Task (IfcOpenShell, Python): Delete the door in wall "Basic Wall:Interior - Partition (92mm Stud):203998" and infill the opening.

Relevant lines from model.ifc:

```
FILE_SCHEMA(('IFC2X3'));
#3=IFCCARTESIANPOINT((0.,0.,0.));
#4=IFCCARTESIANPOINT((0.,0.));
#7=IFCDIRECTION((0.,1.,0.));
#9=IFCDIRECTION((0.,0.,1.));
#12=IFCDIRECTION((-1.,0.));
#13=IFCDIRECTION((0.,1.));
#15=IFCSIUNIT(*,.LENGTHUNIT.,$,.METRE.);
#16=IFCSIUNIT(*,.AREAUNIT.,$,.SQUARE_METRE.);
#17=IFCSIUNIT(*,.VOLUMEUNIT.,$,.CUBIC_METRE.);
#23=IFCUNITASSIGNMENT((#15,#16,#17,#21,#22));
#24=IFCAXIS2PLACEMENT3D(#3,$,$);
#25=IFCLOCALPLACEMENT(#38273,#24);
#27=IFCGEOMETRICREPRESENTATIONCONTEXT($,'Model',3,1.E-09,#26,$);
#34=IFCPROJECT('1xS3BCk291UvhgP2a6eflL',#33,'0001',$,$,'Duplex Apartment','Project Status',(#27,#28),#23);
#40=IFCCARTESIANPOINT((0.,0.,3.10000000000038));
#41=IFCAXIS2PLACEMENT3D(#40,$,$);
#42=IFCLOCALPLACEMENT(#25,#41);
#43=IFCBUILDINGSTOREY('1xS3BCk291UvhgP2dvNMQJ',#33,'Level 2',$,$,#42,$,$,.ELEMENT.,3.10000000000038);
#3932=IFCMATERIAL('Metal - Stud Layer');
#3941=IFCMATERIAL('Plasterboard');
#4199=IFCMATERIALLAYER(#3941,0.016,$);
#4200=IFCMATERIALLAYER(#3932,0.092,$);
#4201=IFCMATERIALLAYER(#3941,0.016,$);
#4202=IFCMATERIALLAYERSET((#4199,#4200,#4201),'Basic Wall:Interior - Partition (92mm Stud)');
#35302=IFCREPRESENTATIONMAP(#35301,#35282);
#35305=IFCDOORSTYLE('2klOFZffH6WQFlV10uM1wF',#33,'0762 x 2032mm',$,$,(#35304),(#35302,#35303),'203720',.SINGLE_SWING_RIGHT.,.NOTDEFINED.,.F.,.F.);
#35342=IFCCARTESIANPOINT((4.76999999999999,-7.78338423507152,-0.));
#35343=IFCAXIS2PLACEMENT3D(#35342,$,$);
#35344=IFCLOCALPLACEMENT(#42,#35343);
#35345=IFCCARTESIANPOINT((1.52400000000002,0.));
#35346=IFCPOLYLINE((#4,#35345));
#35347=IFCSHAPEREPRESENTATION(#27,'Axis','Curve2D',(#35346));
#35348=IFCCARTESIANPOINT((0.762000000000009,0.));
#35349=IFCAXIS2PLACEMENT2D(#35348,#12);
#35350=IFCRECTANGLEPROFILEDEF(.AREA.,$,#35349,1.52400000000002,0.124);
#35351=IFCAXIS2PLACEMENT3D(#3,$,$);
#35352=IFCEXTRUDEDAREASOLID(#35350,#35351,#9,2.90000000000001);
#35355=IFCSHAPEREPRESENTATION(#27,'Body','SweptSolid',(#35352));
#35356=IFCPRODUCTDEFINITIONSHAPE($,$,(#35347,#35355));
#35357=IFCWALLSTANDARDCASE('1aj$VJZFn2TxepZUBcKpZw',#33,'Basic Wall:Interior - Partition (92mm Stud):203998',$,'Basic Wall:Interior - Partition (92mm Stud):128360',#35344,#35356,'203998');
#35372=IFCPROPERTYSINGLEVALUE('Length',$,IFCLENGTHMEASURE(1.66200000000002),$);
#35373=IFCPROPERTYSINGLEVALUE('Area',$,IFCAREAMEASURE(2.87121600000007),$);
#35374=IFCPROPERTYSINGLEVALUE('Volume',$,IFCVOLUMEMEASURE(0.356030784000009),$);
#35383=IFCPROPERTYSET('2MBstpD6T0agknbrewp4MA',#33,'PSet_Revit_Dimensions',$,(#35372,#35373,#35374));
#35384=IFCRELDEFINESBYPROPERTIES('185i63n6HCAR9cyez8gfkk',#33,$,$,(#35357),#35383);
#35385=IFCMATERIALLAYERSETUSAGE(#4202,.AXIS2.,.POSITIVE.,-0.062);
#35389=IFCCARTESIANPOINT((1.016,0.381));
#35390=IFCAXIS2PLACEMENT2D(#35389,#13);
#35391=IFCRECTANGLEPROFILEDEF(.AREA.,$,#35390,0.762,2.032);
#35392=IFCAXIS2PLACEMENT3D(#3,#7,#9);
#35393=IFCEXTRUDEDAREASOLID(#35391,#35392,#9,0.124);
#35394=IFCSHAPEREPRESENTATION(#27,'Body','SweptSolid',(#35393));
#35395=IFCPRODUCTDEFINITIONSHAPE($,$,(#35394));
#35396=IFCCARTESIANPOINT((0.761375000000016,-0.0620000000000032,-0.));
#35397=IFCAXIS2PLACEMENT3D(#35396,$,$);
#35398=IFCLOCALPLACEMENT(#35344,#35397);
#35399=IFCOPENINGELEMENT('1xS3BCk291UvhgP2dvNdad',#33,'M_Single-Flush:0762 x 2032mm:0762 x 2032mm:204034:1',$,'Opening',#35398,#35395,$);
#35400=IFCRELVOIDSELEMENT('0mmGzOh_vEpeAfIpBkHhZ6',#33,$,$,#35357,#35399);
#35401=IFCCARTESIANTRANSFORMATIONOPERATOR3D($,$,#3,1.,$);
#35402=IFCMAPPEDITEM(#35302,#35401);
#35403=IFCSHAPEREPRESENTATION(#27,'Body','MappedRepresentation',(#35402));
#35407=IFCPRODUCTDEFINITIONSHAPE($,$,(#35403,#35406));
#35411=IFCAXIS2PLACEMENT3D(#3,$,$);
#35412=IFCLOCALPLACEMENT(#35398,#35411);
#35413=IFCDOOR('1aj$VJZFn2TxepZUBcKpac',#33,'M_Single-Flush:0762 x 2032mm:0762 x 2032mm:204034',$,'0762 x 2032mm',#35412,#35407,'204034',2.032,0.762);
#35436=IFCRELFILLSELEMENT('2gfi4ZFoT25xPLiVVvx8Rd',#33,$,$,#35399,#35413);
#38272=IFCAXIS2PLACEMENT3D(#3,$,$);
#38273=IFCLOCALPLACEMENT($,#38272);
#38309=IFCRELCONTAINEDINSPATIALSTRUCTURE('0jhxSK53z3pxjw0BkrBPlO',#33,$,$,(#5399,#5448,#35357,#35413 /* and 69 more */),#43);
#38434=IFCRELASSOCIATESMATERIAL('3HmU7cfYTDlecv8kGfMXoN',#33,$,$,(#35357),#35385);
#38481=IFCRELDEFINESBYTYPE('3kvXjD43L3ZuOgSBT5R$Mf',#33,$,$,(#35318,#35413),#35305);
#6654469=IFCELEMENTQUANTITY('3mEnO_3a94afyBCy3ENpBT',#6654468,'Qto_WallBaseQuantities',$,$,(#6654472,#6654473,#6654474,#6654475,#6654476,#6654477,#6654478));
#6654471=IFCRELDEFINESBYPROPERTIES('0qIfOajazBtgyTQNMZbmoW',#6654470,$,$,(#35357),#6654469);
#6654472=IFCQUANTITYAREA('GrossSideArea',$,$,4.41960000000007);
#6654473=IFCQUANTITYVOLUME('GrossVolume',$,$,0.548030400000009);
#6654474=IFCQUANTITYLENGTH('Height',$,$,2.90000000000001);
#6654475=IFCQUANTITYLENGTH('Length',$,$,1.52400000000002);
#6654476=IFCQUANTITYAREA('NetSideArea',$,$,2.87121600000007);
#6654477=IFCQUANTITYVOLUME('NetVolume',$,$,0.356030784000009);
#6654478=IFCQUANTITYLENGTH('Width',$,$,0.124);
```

```python
import ifcopenshell
import ifcopenshell.api.feature
import ifcopenshell.api.pset
import ifcopenshell.api.root
import ifcopenshell.geom
import ifcopenshell.util.element
import ifcopenshell.util.shape
import ifcopenshell.util.unit

model = ifcopenshell.open("model.ifc")
area_scale = ifcopenshell.util.unit.calculate_unit_scale(model, "AREAUNIT")
volume_scale = ifcopenshell.util.unit.calculate_unit_scale(model, "VOLUMEUNIT")
settings = ifcopenshell.geom.settings()


def volume(element):
    """Net volume in cubic metres, openings subtracted."""
    shape = ifcopenshell.geom.create_shape(settings, element)
    return ifcopenshell.util.shape.get_volume(shape.geometry)


door = model.by_guid("1aj$VJZFn2TxepZUBcKpac")
opening = door.FillsVoids[0].RelatingOpeningElement
wall = opening.VoidsElements[0].RelatingBuildingElement
before = volume(wall)

ifcopenshell.api.root.remove_product(model, product=door)
ifcopenshell.api.feature.remove_feature(model, feature=opening)

after = volume(wall)
thickness = 0.124  # wall thickness in metres

# Update the wall's stored quantities.
pset = model.by_id(ifcopenshell.util.element.get_pset(wall, "PSet_Revit_Dimensions", should_inherit=False)["id"])
ifcopenshell.api.pset.edit_pset(model, pset=pset, properties={
    "Area": model.create_entity("IfcAreaMeasure", after / thickness / area_scale),
    "Volume": model.create_entity("IfcVolumeMeasure", after / volume_scale),
})
qto = model.by_id(ifcopenshell.util.element.get_pset(wall, "Qto_WallBaseQuantities", should_inherit=False)["id"])
ifcopenshell.api.pset.edit_qto(model, qto=qto, properties={
    "NetSideArea": after / thickness / area_scale,
    "NetVolume": after / volume_scale,
})

print(f"wall volume {before:.3f} -> {after:.3f} m3")

model.write("model-out.ifc")
```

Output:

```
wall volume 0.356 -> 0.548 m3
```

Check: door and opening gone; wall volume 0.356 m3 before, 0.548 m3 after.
